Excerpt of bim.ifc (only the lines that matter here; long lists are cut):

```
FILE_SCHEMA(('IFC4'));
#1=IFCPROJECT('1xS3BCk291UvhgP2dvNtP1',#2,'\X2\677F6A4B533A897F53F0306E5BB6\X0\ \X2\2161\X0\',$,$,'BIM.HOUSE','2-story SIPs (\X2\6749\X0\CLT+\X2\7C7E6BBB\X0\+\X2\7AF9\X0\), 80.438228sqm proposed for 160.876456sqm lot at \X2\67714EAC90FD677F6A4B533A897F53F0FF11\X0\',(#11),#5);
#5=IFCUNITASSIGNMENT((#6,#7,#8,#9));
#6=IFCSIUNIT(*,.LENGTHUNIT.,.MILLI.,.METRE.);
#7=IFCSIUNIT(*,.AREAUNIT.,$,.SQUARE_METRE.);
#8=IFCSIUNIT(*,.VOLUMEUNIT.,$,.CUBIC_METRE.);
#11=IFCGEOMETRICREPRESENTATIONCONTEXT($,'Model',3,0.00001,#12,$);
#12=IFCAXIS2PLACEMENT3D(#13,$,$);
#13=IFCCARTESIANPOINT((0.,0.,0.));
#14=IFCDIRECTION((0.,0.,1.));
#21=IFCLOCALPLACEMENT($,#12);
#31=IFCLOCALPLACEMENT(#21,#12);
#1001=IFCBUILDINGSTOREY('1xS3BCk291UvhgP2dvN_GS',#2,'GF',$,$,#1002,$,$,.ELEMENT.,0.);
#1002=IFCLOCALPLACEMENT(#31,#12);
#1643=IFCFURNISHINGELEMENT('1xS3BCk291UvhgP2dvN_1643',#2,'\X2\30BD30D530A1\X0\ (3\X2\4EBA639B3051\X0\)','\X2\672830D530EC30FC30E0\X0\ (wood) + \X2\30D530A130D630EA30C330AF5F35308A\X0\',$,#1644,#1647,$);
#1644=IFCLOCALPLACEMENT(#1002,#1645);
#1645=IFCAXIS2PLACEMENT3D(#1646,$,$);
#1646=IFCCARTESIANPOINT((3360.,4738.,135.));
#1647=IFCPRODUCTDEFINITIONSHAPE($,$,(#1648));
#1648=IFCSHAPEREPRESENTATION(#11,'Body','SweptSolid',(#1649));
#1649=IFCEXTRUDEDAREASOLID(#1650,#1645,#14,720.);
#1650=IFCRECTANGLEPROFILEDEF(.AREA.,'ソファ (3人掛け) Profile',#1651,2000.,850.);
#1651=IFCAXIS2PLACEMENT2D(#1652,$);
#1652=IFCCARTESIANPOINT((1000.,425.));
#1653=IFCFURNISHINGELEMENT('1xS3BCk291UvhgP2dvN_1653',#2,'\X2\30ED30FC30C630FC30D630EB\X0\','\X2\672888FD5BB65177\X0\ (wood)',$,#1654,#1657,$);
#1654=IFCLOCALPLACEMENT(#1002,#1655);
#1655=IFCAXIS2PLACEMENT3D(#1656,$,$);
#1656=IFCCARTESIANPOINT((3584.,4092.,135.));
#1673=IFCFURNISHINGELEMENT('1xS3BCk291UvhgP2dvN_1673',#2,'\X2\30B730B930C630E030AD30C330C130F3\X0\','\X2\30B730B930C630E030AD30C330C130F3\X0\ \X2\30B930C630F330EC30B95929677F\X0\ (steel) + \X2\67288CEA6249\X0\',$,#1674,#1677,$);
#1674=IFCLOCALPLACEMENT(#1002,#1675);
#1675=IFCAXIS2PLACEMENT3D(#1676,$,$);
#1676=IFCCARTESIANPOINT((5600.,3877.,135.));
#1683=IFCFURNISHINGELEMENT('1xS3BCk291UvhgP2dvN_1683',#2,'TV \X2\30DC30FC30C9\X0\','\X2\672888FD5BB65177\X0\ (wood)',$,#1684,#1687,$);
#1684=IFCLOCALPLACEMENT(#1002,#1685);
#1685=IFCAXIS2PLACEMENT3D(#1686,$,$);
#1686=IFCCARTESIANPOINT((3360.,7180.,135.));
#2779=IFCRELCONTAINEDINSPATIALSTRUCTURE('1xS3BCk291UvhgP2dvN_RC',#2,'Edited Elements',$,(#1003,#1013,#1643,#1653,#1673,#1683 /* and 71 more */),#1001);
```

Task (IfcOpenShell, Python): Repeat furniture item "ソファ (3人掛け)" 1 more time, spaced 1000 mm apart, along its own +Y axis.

```python
import ifcopenshell
import ifcopenshell.api.geometry
import ifcopenshell.api.root
import ifcopenshell.util.element
import ifcopenshell.util.placement
import ifcopenshell.util.unit

model = ifcopenshell.open("bim.ifc")
unit_scale = ifcopenshell.util.unit.calculate_unit_scale(model)


def reuse_history(source, copy):
    """copy_class also copies each property set's owner history, people and application; keep the originals."""
    for rel in copy.IsDefinedBy:
        if rel.is_a("IfcRelDefinesByProperties") and (history := rel.RelatingPropertyDefinition.OwnerHistory):
            rel.RelatingPropertyDefinition.OwnerHistory = source.OwnerHistory
            ifcopenshell.util.element.remove_deep2(model, history)


source = model.by_guid("1xS3BCk291UvhgP2dvN_1643")
base = ifcopenshell.util.placement.get_local_placement(source.ObjectPlacement)
step = base[:3, 1] * 1 / unit_scale

for i in range(1, 2):
    copy = ifcopenshell.api.root.copy_class(model, product=source)
    copy.Representation = ifcopenshell.util.element.copy_deep(
        model, source.Representation, exclude=["IfcGeometricRepresentationContext", "IfcRepresentationMap"]
    )
    reuse_history(source, copy)
    matrix = base.copy()
    matrix[:3, 3] += i * step
    print("added at", matrix[:3, 3].round(3) + 0.0)
    ifcopenshell.api.geometry.edit_object_placement(model, product=copy, matrix=matrix, is_si=False)

model.write("bim_rev.ifc")
```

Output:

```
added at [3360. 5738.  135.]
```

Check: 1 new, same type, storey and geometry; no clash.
